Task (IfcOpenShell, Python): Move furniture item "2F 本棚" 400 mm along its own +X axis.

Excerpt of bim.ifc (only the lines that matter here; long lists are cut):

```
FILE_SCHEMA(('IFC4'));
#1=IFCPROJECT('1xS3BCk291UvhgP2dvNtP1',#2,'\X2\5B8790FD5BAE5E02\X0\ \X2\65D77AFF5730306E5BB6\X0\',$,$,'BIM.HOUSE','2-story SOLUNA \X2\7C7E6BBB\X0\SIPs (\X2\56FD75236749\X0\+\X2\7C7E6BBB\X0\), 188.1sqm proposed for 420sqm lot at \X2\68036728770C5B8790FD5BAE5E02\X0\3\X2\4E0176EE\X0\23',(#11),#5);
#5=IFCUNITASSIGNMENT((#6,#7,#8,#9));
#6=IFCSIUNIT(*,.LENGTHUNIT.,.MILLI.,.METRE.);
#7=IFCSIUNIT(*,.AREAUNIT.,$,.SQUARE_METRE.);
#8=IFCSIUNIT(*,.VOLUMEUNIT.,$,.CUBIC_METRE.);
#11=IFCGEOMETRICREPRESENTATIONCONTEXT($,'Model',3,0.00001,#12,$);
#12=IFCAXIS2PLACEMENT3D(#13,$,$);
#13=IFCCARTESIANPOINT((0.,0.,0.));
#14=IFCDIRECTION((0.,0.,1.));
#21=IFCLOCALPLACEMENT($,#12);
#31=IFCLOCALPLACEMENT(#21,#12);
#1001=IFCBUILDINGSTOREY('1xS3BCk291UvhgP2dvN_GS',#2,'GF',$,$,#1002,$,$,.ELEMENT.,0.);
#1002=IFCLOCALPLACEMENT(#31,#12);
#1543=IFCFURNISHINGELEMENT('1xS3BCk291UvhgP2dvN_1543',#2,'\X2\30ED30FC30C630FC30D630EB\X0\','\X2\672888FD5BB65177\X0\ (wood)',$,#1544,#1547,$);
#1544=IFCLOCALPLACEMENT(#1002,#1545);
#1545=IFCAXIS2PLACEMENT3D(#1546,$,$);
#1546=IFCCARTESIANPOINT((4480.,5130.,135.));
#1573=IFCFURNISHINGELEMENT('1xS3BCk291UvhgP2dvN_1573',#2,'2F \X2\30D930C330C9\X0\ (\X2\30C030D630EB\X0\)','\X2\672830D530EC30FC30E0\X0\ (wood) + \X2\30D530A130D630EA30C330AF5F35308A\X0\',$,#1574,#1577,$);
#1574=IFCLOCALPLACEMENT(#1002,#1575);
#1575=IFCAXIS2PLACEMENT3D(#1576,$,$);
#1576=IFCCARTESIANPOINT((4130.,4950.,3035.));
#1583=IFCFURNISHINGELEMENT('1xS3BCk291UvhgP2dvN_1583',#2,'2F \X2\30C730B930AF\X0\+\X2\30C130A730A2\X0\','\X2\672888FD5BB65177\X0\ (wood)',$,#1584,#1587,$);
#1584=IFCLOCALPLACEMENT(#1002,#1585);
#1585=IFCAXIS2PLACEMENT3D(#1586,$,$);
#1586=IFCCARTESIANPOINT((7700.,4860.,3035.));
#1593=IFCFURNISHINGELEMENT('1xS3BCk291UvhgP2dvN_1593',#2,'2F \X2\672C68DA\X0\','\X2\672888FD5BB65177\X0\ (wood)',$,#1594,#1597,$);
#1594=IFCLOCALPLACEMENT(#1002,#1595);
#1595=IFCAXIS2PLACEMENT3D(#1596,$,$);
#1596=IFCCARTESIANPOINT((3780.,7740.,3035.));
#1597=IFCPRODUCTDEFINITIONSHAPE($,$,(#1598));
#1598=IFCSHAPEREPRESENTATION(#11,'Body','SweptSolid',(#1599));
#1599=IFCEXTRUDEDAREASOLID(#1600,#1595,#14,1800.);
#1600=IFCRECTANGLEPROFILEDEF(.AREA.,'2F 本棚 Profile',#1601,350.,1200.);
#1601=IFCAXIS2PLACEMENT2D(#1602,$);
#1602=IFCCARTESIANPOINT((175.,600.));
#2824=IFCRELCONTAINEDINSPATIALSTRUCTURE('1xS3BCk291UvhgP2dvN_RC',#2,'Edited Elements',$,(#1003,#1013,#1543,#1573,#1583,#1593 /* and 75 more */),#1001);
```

```python
import ifcopenshell
import ifcopenshell.api.geometry
import ifcopenshell.util.placement

model = ifcopenshell.open("bim.ifc")

item = model.by_id(1593)
matrix = ifcopenshell.util.placement.get_local_placement(item.ObjectPlacement)
matrix[:3, 3] += matrix[:3, 0] * 400.0
ifcopenshell.api.geometry.edit_object_placement(model, product=item, matrix=matrix, is_si=False)

print(ifcopenshell.util.placement.get_local_placement(item.ObjectPlacement).round(3) + 0.0)

model.write("bim_rev.ifc")
```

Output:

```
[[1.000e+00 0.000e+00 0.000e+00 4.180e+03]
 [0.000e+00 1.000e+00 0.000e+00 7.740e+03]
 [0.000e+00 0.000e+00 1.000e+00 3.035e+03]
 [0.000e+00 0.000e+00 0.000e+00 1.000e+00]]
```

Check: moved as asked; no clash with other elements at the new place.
